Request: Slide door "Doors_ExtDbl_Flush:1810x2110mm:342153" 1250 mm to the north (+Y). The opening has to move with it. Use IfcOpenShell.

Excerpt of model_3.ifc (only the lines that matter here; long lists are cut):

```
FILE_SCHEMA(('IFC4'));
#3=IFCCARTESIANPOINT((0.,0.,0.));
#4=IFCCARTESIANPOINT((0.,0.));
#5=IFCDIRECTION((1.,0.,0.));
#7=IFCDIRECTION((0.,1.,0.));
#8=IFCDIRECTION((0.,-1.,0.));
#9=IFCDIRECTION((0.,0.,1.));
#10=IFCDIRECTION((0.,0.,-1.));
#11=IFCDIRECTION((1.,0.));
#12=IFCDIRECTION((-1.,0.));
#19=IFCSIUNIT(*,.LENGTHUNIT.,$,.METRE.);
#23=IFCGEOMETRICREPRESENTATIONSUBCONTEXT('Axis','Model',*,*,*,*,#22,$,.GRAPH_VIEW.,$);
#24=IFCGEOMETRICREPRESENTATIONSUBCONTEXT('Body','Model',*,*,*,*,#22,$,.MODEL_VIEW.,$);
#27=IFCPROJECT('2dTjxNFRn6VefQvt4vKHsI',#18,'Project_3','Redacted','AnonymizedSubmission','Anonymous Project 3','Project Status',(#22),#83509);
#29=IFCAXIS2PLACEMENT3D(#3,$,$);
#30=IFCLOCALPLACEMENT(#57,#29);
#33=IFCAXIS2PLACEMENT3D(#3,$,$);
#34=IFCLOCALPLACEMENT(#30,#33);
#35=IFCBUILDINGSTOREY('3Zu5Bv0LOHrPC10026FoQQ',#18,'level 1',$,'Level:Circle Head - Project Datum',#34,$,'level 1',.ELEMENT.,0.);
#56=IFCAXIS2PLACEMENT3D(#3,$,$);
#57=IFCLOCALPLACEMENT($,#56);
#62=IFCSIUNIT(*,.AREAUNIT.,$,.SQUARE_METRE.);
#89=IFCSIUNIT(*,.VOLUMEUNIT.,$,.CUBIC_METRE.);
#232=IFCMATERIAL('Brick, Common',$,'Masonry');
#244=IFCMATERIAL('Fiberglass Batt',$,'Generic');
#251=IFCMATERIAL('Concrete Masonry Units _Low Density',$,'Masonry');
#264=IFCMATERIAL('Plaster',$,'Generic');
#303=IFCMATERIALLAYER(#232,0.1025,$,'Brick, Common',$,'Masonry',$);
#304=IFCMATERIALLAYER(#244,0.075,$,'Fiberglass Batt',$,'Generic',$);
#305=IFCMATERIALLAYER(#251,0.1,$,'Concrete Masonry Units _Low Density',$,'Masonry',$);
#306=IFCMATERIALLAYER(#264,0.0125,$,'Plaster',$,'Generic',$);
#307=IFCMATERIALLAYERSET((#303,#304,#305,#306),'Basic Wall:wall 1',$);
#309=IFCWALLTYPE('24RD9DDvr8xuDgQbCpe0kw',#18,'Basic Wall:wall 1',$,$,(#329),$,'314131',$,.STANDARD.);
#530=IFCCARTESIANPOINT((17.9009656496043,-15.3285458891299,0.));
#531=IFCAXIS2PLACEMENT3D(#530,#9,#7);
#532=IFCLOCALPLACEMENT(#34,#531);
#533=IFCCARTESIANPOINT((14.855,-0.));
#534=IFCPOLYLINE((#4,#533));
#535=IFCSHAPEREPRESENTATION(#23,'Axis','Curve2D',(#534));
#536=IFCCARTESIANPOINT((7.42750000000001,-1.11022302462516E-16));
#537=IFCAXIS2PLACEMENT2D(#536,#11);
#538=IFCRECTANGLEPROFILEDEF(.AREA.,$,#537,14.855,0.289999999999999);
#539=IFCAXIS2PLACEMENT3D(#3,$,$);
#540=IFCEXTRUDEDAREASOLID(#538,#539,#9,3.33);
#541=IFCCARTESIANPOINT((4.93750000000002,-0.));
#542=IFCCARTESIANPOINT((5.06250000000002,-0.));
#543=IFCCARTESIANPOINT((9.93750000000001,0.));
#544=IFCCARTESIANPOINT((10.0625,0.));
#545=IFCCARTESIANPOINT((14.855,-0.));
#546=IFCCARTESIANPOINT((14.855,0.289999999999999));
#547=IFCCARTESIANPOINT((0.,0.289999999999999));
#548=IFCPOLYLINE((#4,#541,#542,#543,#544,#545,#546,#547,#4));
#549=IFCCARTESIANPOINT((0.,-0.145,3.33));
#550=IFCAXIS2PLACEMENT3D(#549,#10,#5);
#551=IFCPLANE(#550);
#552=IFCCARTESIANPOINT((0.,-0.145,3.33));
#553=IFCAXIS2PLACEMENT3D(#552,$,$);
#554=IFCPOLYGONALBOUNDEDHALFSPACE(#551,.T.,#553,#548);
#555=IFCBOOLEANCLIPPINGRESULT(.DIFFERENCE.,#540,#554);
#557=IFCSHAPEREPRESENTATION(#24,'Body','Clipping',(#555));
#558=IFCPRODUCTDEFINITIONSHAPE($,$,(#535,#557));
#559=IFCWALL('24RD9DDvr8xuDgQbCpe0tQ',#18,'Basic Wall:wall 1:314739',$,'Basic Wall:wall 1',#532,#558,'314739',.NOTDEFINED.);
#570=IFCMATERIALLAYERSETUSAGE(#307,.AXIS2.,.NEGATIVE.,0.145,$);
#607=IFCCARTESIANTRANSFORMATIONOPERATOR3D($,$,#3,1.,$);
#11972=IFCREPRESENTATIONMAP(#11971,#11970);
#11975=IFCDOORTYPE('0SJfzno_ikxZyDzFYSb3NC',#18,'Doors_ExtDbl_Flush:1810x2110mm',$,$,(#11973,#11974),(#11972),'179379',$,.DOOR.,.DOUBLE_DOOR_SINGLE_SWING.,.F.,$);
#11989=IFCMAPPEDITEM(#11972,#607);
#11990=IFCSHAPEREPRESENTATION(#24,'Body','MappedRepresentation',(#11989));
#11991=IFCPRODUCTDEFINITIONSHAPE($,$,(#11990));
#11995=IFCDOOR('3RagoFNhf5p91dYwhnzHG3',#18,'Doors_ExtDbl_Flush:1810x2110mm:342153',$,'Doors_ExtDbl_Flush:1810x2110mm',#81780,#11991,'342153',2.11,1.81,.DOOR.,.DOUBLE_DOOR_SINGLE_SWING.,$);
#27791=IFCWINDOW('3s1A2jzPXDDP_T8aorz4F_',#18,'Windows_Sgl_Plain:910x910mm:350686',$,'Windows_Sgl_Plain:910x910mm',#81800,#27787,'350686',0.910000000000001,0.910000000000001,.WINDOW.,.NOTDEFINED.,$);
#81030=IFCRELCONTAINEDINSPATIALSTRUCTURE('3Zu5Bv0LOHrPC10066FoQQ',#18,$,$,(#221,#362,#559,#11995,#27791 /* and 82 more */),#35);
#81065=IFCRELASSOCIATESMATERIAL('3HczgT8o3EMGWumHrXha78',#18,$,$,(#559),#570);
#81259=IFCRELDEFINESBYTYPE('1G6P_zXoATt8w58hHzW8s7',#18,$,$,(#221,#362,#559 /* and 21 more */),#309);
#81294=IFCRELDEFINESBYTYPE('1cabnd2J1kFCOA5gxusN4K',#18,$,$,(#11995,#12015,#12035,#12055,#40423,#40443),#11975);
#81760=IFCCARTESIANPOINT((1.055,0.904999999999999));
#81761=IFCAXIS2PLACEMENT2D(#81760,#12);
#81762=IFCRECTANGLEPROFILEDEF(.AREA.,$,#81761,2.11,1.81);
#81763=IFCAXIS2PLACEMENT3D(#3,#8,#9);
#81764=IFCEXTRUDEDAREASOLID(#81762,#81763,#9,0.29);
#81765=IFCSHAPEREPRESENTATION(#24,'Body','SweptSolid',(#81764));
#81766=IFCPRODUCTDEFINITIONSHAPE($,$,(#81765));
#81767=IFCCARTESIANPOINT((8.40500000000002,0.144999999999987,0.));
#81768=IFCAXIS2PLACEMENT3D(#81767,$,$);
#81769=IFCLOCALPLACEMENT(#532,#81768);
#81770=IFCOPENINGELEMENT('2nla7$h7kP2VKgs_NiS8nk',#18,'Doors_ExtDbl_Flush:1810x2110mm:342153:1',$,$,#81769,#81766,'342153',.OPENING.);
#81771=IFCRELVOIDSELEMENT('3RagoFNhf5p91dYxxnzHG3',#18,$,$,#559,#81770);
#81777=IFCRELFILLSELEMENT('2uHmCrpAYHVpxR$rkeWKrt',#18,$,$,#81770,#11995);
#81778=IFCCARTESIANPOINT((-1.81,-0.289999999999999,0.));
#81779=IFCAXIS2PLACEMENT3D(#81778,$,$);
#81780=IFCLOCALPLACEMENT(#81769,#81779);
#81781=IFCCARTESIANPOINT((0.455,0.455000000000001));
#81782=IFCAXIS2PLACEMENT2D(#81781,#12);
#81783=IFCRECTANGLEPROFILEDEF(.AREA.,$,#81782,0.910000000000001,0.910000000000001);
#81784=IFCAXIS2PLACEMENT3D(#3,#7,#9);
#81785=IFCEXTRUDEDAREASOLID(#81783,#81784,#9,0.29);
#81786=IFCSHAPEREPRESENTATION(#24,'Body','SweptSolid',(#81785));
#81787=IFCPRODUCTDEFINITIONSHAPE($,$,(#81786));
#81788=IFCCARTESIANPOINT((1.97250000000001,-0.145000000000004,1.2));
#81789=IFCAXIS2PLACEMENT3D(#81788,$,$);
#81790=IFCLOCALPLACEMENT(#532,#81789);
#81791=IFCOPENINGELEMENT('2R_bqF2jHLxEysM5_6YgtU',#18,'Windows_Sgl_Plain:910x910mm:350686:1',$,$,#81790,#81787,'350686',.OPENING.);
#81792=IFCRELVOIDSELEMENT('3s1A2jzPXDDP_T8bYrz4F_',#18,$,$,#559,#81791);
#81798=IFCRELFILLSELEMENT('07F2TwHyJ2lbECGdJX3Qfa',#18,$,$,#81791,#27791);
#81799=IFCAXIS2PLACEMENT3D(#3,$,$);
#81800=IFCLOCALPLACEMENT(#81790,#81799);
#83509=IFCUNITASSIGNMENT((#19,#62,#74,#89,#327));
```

```python
import ifcopenshell
import ifcopenshell.api.geometry
import ifcopenshell.util.placement
import ifcopenshell.util.unit

model = ifcopenshell.open("model_3.ifc")
unit_scale = ifcopenshell.util.unit.calculate_unit_scale(model)

door = model.by_id(11995)
opening = door.FillsVoids[0].RelatingOpeningElement
wall = opening.VoidsElements[0].RelatingBuildingElement

wall_matrix = ifcopenshell.util.placement.get_local_placement(wall.ObjectPlacement)
shift = wall_matrix[:3, 0] * 1.25 / unit_scale
before = ifcopenshell.util.placement.get_local_placement(door.ObjectPlacement)[:3, 3].copy()

# The door is placed relative to its opening, so it follows when the opening moves.
matrix = ifcopenshell.util.placement.get_local_placement(opening.ObjectPlacement)
matrix[:3, 3] += shift
ifcopenshell.api.geometry.edit_object_placement(
    model, product=opening, matrix=matrix, is_si=False, should_transform_children=True
)

after = ifcopenshell.util.placement.get_local_placement(door.ObjectPlacement)[:3, 3]
print("door moved by", (after - before).round(3) + 0.0)

model.write("model_3_updated.ifc")
```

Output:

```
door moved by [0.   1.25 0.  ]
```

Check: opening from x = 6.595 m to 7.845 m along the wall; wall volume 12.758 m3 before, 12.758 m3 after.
